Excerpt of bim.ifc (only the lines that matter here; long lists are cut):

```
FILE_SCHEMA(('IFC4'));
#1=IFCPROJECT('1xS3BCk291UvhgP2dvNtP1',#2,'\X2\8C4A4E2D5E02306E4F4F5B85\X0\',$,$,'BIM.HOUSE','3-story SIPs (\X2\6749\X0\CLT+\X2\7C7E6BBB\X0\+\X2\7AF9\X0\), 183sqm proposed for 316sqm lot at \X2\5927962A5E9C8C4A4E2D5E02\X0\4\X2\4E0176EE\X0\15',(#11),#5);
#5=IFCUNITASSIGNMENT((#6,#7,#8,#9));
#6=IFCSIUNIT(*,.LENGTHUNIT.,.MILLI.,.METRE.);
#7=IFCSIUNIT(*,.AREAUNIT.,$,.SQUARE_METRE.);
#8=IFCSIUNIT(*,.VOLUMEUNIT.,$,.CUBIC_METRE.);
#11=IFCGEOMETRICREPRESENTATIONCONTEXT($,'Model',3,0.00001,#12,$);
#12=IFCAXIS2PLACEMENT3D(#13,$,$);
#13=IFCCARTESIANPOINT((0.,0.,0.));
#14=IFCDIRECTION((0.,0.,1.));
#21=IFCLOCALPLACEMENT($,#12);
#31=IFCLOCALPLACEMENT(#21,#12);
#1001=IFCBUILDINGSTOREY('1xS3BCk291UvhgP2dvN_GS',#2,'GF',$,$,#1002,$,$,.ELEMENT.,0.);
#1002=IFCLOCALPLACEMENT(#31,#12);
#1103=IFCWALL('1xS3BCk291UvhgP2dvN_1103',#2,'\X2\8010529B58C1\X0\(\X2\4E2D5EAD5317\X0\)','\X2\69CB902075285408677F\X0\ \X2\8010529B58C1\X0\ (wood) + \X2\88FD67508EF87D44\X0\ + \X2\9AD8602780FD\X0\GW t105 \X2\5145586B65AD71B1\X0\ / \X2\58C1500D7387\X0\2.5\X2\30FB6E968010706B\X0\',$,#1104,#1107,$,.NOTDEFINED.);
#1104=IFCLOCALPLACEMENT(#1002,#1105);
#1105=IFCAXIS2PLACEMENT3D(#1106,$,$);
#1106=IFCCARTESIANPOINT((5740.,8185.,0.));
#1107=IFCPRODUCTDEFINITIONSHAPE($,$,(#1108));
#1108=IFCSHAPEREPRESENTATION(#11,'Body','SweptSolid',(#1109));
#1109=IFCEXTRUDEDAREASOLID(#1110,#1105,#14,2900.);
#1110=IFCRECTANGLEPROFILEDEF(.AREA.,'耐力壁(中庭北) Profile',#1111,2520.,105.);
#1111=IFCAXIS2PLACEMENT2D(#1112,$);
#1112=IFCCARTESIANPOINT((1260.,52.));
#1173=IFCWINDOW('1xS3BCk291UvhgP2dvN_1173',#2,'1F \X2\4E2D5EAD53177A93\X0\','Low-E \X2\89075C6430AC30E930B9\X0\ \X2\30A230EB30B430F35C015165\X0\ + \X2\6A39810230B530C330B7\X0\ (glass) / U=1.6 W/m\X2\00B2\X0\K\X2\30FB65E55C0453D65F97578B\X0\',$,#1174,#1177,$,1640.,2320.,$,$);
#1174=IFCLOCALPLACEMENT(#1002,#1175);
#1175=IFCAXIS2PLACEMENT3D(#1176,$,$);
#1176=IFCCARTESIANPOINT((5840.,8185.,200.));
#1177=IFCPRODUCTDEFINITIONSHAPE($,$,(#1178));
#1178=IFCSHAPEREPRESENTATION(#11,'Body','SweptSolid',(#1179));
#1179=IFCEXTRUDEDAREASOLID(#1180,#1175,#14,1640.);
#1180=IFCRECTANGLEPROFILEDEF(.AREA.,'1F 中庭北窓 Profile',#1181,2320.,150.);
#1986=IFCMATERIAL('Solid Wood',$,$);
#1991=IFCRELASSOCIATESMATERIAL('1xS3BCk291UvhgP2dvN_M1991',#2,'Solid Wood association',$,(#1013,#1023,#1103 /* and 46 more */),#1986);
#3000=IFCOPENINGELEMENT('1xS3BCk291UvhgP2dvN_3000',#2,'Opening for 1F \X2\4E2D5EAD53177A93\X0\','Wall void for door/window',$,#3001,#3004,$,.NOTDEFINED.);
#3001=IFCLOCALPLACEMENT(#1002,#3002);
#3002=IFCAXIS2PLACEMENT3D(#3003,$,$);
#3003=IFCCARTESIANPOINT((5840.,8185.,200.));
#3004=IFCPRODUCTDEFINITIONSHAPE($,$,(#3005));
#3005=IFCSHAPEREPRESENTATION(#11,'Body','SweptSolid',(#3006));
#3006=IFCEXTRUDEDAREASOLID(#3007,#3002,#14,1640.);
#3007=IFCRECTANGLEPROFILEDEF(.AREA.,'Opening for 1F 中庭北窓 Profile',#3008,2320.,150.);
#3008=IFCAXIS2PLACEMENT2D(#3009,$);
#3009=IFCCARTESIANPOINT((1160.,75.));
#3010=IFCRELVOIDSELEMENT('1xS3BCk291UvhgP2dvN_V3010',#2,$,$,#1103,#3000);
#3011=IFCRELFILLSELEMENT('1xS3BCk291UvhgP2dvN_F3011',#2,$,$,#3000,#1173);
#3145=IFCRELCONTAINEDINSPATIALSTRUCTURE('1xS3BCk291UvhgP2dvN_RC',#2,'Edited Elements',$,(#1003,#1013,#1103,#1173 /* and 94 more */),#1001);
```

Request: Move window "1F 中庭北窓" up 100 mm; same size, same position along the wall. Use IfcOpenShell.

```python
import numpy as np
import ifcopenshell
import ifcopenshell.api.geometry
import ifcopenshell.util.placement
import ifcopenshell.util.unit

model = ifcopenshell.open("bim.ifc")
unit_scale = ifcopenshell.util.unit.calculate_unit_scale(model)

window = model.by_id(1173)
opening = window.FillsVoids[0].RelatingOpeningElement
dz = 0.1 / unit_scale

shift = np.array([0.0, 0.0, dz])
# The window is not placed relative to its opening, so move both.
for product in (opening, window):
    matrix = ifcopenshell.util.placement.get_local_placement(product.ObjectPlacement)
    matrix[:3, 3] += shift
    ifcopenshell.api.geometry.edit_object_placement(model, product=product, matrix=matrix, is_si=False)

print(f"moved by {dz * unit_scale:+.3f} m")

model.write("bim-out.ifc")
```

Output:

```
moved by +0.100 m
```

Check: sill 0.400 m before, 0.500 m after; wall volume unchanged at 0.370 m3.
